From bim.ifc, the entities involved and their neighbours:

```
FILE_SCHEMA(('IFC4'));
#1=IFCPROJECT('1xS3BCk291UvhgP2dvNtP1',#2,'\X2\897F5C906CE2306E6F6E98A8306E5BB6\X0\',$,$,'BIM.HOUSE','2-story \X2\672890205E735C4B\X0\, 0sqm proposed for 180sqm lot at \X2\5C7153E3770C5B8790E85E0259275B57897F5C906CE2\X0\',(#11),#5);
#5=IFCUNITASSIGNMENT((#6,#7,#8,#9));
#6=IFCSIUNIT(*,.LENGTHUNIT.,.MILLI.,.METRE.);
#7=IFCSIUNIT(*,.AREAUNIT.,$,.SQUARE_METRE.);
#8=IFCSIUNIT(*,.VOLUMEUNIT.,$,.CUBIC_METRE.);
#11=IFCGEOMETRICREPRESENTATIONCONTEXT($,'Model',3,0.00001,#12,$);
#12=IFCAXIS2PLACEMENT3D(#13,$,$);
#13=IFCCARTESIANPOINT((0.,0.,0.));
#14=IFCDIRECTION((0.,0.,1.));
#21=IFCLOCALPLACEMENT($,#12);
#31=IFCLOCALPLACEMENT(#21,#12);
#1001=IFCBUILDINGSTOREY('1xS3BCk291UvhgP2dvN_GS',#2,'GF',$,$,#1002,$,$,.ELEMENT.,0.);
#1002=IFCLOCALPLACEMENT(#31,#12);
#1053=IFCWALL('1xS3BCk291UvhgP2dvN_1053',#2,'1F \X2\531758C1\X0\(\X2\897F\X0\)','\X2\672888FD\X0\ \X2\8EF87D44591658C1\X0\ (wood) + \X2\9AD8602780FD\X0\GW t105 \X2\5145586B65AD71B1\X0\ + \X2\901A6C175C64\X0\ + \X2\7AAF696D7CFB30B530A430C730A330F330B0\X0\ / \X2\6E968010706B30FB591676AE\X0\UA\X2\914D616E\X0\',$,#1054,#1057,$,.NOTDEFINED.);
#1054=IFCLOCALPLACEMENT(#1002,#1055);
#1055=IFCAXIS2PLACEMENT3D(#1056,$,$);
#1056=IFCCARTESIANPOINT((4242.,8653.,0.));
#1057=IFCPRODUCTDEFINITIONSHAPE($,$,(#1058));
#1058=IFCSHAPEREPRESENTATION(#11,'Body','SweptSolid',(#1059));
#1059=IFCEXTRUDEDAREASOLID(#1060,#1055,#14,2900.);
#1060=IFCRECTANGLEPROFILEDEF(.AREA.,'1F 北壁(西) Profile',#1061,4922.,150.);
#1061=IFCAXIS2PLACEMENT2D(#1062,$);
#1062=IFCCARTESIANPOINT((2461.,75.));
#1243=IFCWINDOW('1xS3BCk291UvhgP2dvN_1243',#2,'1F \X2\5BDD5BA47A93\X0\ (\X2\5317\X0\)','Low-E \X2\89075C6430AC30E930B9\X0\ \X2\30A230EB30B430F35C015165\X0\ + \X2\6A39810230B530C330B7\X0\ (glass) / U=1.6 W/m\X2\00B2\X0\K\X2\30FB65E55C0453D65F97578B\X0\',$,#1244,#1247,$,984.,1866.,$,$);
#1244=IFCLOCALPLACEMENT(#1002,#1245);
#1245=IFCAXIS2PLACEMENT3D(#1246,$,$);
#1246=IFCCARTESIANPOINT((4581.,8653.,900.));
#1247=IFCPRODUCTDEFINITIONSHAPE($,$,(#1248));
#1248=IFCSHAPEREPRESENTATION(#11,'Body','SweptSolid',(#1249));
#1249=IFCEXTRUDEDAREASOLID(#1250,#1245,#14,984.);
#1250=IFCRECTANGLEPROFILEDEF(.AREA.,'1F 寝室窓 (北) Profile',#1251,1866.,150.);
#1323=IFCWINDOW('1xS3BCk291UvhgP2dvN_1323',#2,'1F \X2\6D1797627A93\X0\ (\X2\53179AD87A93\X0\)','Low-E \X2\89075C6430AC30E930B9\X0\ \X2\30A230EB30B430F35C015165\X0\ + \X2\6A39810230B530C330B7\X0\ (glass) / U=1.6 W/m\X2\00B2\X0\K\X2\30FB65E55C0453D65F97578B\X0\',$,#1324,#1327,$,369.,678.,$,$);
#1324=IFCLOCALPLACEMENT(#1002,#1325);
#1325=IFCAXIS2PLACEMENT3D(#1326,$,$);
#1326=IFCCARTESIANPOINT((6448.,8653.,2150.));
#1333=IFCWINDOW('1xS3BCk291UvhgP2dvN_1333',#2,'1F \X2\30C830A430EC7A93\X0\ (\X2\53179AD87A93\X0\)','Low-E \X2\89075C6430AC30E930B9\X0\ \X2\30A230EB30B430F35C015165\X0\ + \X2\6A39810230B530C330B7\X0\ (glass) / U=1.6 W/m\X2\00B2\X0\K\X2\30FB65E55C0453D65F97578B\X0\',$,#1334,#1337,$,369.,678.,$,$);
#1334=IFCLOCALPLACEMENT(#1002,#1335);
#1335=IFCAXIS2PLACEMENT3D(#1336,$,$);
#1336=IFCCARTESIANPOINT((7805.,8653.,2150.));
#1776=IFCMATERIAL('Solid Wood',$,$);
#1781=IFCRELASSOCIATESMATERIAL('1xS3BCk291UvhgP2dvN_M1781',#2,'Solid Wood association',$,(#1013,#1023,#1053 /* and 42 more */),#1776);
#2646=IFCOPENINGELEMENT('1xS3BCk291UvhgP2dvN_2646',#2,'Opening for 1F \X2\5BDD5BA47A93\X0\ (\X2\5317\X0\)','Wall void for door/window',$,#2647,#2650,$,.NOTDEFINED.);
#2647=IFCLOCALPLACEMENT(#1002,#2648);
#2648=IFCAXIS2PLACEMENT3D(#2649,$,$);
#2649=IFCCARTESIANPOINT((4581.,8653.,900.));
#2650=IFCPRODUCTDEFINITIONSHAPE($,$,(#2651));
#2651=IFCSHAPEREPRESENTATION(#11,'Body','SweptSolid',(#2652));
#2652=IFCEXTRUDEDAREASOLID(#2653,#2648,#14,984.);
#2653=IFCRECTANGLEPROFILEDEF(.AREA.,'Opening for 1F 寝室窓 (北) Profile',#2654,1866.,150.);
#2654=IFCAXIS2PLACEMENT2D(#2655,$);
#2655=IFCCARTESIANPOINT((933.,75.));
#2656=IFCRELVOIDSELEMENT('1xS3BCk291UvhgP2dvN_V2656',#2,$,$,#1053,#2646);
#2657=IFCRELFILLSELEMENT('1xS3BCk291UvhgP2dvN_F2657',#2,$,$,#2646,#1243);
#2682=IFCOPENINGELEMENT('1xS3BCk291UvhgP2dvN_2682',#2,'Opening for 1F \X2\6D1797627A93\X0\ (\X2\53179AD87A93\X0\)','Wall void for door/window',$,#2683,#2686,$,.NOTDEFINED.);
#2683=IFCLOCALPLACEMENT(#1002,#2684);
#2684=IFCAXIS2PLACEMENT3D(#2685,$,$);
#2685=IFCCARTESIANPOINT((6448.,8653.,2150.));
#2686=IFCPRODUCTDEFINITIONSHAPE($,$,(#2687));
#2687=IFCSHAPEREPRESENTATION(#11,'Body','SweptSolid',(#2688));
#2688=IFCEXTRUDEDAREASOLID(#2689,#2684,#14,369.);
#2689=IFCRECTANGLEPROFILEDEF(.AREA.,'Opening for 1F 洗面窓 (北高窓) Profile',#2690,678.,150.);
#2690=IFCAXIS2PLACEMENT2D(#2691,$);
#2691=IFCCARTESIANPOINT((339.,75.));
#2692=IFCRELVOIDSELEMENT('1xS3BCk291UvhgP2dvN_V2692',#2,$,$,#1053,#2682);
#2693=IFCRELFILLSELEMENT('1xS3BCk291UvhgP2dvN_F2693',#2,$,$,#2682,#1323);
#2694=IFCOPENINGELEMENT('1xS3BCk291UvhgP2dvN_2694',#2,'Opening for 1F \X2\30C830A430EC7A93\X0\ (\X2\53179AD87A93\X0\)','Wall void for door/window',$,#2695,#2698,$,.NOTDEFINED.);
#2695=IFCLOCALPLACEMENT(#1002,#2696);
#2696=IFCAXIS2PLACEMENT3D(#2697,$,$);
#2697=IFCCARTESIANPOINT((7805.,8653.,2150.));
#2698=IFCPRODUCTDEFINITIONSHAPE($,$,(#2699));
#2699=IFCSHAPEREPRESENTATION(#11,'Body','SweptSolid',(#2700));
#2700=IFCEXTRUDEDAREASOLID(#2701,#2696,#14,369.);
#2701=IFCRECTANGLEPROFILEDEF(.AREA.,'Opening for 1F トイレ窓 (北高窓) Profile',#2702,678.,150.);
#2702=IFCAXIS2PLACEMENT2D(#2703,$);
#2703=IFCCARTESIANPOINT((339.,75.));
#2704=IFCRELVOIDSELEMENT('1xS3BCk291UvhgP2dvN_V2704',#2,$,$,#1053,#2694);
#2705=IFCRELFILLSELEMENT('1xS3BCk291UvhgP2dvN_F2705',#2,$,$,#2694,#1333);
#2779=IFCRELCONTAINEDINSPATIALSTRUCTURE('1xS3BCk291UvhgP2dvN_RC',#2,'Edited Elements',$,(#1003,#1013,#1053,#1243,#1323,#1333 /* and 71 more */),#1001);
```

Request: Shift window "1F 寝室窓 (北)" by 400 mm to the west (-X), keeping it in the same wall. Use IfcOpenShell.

```python
import ifcopenshell
import ifcopenshell.api.geometry
import ifcopenshell.util.placement
import ifcopenshell.util.unit

model = ifcopenshell.open("bim.ifc")
unit_scale = ifcopenshell.util.unit.calculate_unit_scale(model)

window = model.by_id(1243)
opening = window.FillsVoids[0].RelatingOpeningElement
wall = opening.VoidsElements[0].RelatingBuildingElement

wall_matrix = ifcopenshell.util.placement.get_local_placement(wall.ObjectPlacement)
shift = wall_matrix[:3, 0] * -0.4 / unit_scale
before = ifcopenshell.util.placement.get_local_placement(window.ObjectPlacement)[:3, 3].copy()

# The window is not placed relative to its opening, so move both.
for product in (opening, window):
    matrix = ifcopenshell.util.placement.get_local_placement(product.ObjectPlacement)
    matrix[:3, 3] += shift
    ifcopenshell.api.geometry.edit_object_placement(model, product=product, matrix=matrix, is_si=False)

after = ifcopenshell.util.placement.get_local_placement(window.ObjectPlacement)[:3, 3]
print("window moved by", (after - before).round(3) + 0.0)

model.write("bim_updated.ifc")
```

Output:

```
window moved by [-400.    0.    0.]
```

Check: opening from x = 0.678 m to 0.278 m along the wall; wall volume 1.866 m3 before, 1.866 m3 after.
